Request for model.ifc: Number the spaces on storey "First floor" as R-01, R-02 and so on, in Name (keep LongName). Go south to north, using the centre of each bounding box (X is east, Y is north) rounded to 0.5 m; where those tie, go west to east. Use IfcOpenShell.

First a look at what the model holds.

```python
import ifcopenshell
import ifcopenshell.util.element
import ifcopenshell.util.placement

model = ifcopenshell.open("model.ifc")
print(model.schema)
storey = next(s for s in model.by_type("IfcBuildingStorey") if s.Name == "First floor")
spaces = [e for e in ifcopenshell.util.element.get_decomposition(storey) if e.is_a("IfcSpace")]
for e in sorted(spaces, key=lambda e: e.id()):
    origin = ifcopenshell.util.placement.get_local_placement(e.ObjectPlacement)[:3, 3]
    print(e.id(), e.Name, e.LongName, origin.round(2) + 0.0, sep=" | ")
```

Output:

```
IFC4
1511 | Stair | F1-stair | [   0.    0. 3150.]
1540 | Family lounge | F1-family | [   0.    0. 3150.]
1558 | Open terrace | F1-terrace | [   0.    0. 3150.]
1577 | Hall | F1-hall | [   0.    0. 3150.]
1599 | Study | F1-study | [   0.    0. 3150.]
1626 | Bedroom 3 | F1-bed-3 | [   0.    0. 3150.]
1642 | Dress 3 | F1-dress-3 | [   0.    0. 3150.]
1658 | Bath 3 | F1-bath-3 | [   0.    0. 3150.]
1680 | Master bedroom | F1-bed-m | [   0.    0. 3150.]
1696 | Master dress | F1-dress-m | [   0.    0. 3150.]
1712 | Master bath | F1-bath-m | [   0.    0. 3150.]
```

```python
import ifcopenshell
import ifcopenshell.geom
import ifcopenshell.util.element
import ifcopenshell.util.shape

model = ifcopenshell.open("model.ifc")
settings = ifcopenshell.geom.settings()
settings.set("use-world-coords", True)


def centre(element):
    shape = ifcopenshell.geom.create_shape(settings, element)
    return ifcopenshell.util.shape.get_bbox_centroid(shape.geometry)


storey = next(s for s in model.by_type("IfcBuildingStorey") if s.Name == "First floor")
spaces = [e for e in ifcopenshell.util.element.get_decomposition(storey) if e.is_a("IfcSpace")]

# Insertion points can sit at a corner or the storey origin, so sort by the geometry (in metres).
centres = {e: centre(e) for e in spaces}
spaces.sort(key=lambda e: (round(centres[e][1] / 0.5), centres[e][0]))

for i, e in enumerate(spaces, start=1):
    number = f"R-{i:02d}"
    e.Name = number
    print(e.id(), number)

model.write("model_updated.ifc")
```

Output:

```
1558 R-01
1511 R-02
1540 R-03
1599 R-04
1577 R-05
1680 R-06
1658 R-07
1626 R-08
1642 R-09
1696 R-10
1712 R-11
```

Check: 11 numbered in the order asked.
